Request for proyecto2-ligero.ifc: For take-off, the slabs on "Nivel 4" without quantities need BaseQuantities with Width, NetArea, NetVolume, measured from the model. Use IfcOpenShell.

First a look at what the model holds.

```python
import ifcopenshell
import ifcopenshell.util.element
import ifcopenshell.util.unit

model = ifcopenshell.open("proyecto2-ligero.ifc")
print(model.schema)
for unit_type in ("LENGTHUNIT", "AREAUNIT", "VOLUMEUNIT"):
    print(unit_type, ifcopenshell.util.unit.calculate_unit_scale(model, unit_type))
storey = next(s for s in model.by_type("IfcBuildingStorey") if s.Name == "Nivel 4")
slabs = [e for e in ifcopenshell.util.element.get_decomposition(storey) if e.is_a("IfcSlab")]
for e in sorted(slabs, key=lambda e: e.id()):
    print(e.id(), e.is_a(), e.Name, list(ifcopenshell.util.element.get_psets(e, qtos_only=True)), sep=" | ")
```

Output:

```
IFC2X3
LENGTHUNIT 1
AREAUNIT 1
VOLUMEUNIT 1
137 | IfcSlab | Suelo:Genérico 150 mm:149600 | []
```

```python
import ifcopenshell
import ifcopenshell.api.pset
import ifcopenshell.geom
import ifcopenshell.util.element
import ifcopenshell.util.shape
import ifcopenshell.util.unit

model = ifcopenshell.open("proyecto2-ligero.ifc")
unit_scale = ifcopenshell.util.unit.calculate_unit_scale(model)
area_scale = ifcopenshell.util.unit.calculate_unit_scale(model, "AREAUNIT")
volume_scale = ifcopenshell.util.unit.calculate_unit_scale(model, "VOLUMEUNIT")
settings = ifcopenshell.geom.settings()

storey = next(s for s in model.by_type("IfcBuildingStorey") if s.Name == "Nivel 4")
slabs = [e for e in ifcopenshell.util.element.get_decomposition(storey) if e.is_a("IfcSlab")]

for e in sorted(slabs, key=lambda e: e.id()):
    if ifcopenshell.util.element.get_psets(e, qtos_only=True, should_inherit=False):
        continue
    # Geometry comes back in metres, in the element's own axes.
    shape = ifcopenshell.geom.create_shape(settings, e)
    values = {
        "Width": ifcopenshell.util.shape.get_z(shape.geometry) / unit_scale,
        "NetArea": ifcopenshell.util.shape.get_footprint_area(shape.geometry) / area_scale,
        "NetVolume": ifcopenshell.util.shape.get_volume(shape.geometry) / volume_scale,
    }
    qto = ifcopenshell.api.pset.add_qto(model, product=e, name="BaseQuantities")
    ifcopenshell.api.pset.edit_qto(model, qto=qto, properties=values)
    print(e.id(), {k: round(v, 3) for k, v in values.items()})

model.write("proyecto2-ligero_edited.ifc")
```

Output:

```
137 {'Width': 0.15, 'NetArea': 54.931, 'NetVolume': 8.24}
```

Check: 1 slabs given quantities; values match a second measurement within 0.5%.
